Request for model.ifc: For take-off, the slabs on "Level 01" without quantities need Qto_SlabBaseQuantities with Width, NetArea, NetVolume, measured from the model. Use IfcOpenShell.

First a look at what the model holds.

```python
import ifcopenshell
import ifcopenshell.util.element
import ifcopenshell.util.unit

model = ifcopenshell.open("model.ifc")
print(model.schema)
for unit_type in ("LENGTHUNIT", "AREAUNIT", "VOLUMEUNIT"):
    print(unit_type, ifcopenshell.util.unit.calculate_unit_scale(model, unit_type))
storey = next(s for s in model.by_type("IfcBuildingStorey") if s.Name == "Level 01")
slabs = [e for e in ifcopenshell.util.element.get_decomposition(storey) if e.is_a("IfcSlab")]
for e in sorted(slabs, key=lambda e: e.id()):
    print(e.id(), e.is_a(), e.Name, list(ifcopenshell.util.element.get_psets(e, qtos_only=True)), sep=" | ")
```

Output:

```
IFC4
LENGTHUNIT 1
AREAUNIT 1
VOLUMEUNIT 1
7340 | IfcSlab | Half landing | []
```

```python
import ifcopenshell
import ifcopenshell.api.pset
import ifcopenshell.geom
import ifcopenshell.util.element
import ifcopenshell.util.shape
import ifcopenshell.util.unit

model = ifcopenshell.open("model.ifc")
unit_scale = ifcopenshell.util.unit.calculate_unit_scale(model)
area_scale = ifcopenshell.util.unit.calculate_unit_scale(model, "AREAUNIT")
volume_scale = ifcopenshell.util.unit.calculate_unit_scale(model, "VOLUMEUNIT")
settings = ifcopenshell.geom.settings()

storey = next(s for s in model.by_type("IfcBuildingStorey") if s.Name == "Level 01")
slabs = [e for e in ifcopenshell.util.element.get_decomposition(storey) if e.is_a("IfcSlab")]

for e in sorted(slabs, key=lambda e: e.id()):
    if ifcopenshell.util.element.get_psets(e, qtos_only=True, should_inherit=False):
        continue
    # Geometry comes back in metres, in the element's own axes.
    shape = ifcopenshell.geom.create_shape(settings, e)
    values = {
        "Width": ifcopenshell.util.shape.get_z(shape.geometry) / unit_scale,
        "NetArea": ifcopenshell.util.shape.get_footprint_area(shape.geometry) / area_scale,
        "NetVolume": ifcopenshell.util.shape.get_volume(shape.geometry) / volume_scale,
    }
    qto = ifcopenshell.api.pset.add_qto(model, product=e, name="Qto_SlabBaseQuantities")
    ifcopenshell.api.pset.edit_qto(model, qto=qto, properties=values)
    print(e.id(), {k: round(v, 3) for k, v in values.items()})

model.write("model_edited.ifc")
```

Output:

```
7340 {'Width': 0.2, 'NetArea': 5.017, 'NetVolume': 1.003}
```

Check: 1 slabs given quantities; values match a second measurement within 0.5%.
